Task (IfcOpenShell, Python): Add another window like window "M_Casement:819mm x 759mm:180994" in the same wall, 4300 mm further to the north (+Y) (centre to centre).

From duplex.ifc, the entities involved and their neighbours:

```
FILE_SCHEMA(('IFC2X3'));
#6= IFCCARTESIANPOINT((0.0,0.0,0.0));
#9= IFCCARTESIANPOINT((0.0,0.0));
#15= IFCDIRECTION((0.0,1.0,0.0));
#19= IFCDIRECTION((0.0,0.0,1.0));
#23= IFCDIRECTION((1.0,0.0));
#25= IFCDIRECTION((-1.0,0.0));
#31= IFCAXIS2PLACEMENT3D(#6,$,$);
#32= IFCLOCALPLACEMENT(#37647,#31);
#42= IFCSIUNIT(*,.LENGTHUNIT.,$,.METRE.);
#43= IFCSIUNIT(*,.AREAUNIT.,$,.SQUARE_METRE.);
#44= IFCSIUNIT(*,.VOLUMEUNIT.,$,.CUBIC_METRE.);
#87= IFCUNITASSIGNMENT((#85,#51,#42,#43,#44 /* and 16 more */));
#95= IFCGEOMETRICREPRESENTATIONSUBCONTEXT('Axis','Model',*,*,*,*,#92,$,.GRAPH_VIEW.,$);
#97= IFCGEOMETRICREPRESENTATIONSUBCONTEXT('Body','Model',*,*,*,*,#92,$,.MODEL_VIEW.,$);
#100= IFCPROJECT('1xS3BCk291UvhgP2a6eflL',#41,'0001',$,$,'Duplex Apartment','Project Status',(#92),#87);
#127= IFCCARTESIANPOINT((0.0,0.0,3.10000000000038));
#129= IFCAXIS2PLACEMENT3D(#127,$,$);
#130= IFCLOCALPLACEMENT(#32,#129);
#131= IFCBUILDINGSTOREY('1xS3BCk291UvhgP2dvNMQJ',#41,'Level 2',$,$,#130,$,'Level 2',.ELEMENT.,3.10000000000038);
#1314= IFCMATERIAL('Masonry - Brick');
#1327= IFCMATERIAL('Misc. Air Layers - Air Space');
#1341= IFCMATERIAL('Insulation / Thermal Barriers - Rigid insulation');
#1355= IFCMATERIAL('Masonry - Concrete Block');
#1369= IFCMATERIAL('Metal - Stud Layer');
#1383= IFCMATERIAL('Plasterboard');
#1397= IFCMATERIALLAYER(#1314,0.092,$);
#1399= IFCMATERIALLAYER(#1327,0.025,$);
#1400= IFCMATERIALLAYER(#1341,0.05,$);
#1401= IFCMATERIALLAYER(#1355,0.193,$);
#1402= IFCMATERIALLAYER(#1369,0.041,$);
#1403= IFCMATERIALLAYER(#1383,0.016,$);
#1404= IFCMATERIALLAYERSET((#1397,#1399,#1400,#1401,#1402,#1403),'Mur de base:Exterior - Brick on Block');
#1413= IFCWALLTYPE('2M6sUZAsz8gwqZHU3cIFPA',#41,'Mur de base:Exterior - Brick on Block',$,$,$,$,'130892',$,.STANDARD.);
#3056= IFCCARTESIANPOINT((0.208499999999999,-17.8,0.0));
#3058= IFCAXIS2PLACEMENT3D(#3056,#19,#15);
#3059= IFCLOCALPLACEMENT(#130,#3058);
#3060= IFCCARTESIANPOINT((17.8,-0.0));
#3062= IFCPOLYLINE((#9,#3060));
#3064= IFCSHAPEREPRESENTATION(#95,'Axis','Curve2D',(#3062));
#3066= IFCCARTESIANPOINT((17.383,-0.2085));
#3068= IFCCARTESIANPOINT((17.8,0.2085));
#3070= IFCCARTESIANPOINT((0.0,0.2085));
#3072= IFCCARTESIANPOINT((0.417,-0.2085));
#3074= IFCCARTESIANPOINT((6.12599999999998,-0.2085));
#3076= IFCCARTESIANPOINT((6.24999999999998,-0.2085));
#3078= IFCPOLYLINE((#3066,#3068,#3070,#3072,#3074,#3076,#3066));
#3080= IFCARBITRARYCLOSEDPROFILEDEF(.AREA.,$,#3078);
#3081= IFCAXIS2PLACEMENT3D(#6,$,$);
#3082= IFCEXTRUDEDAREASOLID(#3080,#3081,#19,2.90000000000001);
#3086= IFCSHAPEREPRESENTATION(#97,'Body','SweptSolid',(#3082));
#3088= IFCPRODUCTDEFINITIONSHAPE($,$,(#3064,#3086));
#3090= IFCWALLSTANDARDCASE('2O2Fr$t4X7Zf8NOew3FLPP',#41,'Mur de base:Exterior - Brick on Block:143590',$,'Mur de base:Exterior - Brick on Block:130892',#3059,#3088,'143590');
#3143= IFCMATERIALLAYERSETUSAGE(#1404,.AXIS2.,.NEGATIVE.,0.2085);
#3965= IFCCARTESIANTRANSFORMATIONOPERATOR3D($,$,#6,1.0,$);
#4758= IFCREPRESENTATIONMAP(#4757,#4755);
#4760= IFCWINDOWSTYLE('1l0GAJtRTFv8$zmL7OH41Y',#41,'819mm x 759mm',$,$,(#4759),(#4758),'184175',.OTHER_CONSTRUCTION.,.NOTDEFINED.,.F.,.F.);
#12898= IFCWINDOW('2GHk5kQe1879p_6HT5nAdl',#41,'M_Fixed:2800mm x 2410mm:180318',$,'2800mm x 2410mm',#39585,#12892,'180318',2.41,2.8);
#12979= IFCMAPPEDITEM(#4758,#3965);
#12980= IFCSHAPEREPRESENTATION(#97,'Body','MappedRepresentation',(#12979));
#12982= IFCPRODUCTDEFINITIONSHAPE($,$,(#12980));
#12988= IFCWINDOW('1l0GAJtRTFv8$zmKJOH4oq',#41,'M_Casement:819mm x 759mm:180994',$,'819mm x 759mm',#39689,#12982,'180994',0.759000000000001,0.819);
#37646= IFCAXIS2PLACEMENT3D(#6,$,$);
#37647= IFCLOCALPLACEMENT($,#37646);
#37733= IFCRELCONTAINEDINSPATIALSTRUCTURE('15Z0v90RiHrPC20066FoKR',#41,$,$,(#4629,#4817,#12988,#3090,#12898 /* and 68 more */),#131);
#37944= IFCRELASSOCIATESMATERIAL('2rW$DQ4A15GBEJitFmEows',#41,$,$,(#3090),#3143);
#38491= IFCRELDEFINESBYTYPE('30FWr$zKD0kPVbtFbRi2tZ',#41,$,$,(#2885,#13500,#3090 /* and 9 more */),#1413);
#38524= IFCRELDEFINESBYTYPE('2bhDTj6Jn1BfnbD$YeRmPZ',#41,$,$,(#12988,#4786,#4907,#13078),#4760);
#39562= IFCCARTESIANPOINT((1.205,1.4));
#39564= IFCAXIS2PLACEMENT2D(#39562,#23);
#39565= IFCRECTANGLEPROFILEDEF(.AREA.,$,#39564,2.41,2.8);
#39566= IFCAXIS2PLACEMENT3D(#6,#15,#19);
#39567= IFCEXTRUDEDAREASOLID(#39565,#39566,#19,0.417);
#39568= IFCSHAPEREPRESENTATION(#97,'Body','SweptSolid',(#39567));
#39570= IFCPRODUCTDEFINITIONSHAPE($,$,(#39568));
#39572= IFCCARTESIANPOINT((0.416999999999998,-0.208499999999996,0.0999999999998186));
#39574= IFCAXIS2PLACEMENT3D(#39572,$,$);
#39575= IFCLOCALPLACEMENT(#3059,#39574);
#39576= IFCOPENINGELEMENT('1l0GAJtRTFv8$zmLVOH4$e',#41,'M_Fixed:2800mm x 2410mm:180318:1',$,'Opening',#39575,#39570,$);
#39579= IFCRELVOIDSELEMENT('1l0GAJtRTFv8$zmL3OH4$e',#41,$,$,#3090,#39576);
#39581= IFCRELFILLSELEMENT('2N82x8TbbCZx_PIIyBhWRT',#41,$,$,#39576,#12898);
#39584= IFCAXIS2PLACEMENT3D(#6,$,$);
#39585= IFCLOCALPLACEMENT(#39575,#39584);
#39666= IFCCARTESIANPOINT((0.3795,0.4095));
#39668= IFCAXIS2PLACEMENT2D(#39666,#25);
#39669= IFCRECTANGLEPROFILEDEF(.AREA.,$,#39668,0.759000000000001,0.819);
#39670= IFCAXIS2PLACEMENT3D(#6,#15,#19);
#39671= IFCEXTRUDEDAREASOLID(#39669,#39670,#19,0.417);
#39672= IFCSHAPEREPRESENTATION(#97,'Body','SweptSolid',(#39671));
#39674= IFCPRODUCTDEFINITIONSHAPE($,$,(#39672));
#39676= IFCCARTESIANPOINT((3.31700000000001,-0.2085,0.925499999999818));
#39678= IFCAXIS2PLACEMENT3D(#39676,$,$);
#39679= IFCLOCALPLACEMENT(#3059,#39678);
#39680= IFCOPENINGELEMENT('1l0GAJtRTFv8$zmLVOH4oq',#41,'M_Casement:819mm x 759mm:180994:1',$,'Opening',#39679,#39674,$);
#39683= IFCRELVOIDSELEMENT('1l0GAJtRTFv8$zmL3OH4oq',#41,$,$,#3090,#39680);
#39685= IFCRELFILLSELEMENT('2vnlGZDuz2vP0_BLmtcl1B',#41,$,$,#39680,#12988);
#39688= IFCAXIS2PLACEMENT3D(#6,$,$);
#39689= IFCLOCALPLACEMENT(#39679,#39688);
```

```python
import ifcopenshell
import ifcopenshell.api.feature
import ifcopenshell.api.geometry
import ifcopenshell.api.root
import ifcopenshell.geom
import ifcopenshell.util.element
import ifcopenshell.util.placement
import ifcopenshell.util.shape

model = ifcopenshell.open("duplex.ifc")
settings = ifcopenshell.geom.settings()


def volume(element):
    """Net volume in cubic metres, openings subtracted."""
    shape = ifcopenshell.geom.create_shape(settings, element)
    return ifcopenshell.util.shape.get_volume(shape.geometry)


def reuse_history(source, copy):
    """copy_class also copies each property set's owner history, people and application; keep the originals."""
    for rel in copy.IsDefinedBy:
        if rel.is_a("IfcRelDefinesByProperties") and (history := rel.RelatingPropertyDefinition.OwnerHistory):
            rel.RelatingPropertyDefinition.OwnerHistory = source.OwnerHistory
            ifcopenshell.util.element.remove_deep2(model, history)


window = model.by_id(12988)
opening = window.FillsVoids[0].RelatingOpeningElement
wall = opening.VoidsElements[0].RelatingBuildingElement
before = volume(wall)
shift = ifcopenshell.util.placement.get_local_placement(wall.ObjectPlacement)[:3, 0] * 4.3

# copy_class copies the void relationship, type, container and properties, but no geometry.
new_opening = ifcopenshell.api.root.copy_class(model, product=opening)
new_opening.Representation = ifcopenshell.util.element.copy_deep(
    model, opening.Representation, exclude=["IfcGeometricRepresentationContext", "IfcRepresentationMap"]
)
new_opening.Name = "M_Casement:819mm x 759mm"
new_window = ifcopenshell.api.root.copy_class(model, product=window)
new_window.Representation = ifcopenshell.util.element.copy_deep(
    model, window.Representation, exclude=["IfcGeometricRepresentationContext", "IfcRepresentationMap"]
)
new_window.Name = "M_Casement:819mm x 759mm"
new_window.Tag = None
reuse_history(window, new_window)
fills = ifcopenshell.api.feature.add_filling(model, opening=new_opening, element=new_window)
fills.OwnerHistory = new_window.OwnerHistory  # required in IFC2X3

for old, new in ((opening, new_opening), (window, new_window)):
    matrix = ifcopenshell.util.placement.get_local_placement(old.ObjectPlacement)
    matrix[:3, 3] += shift
    ifcopenshell.api.geometry.edit_object_placement(model, product=new, matrix=matrix, is_si=False)

after = volume(wall)

print(f"wall volume {before:.3f} -> {after:.3f} m3")

model.write("duplex_edited.ifc")
```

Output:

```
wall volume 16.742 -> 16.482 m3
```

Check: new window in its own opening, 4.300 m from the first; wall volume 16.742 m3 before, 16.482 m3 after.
